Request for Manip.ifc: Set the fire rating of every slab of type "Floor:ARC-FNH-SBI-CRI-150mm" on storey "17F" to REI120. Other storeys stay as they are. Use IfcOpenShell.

First a look at what the model holds.

```python
import ifcopenshell
import ifcopenshell.util.element

model = ifcopenshell.open("Manip.ifc")
print(model.schema)
storey = next(s for s in model.by_type("IfcBuildingStorey") if s.Name == "17F")
slabs = [e for e in ifcopenshell.util.element.get_decomposition(storey) if e.is_a("IfcSlab")]
seen = {}
for e in slabs:
    element_type = ifcopenshell.util.element.get_type(e)
    key = (element_type.Name if element_type != e and element_type else None, ifcopenshell.util.element.get_pset(e, "Pset_SlabCommon", "FireRating"))
    seen[key] = seen.get(key, 0) + 1
for (name, value), count in sorted(seen.items(), key=str):
    print(count, "x", name, "|", value)
```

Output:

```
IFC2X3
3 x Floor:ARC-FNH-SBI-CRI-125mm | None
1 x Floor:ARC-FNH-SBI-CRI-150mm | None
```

```python
import ifcopenshell
import ifcopenshell.api.pset
import ifcopenshell.util.element

model = ifcopenshell.open("Manip.ifc")

storey = next(s for s in model.by_type("IfcBuildingStorey") if s.Name == "17F")
slabs = [e for e in ifcopenshell.util.element.get_decomposition(storey) if e.is_a("IfcSlab")]

count = 0
for e in slabs:
    element_type = ifcopenshell.util.element.get_type(e)
    if element_type in (None, e) or element_type.Name != "Floor:ARC-FNH-SBI-CRI-150mm":
        continue
    # add_pset returns the element's existing set when there is one.
    pset = ifcopenshell.api.pset.add_pset(model, product=e, name="Pset_SlabCommon")
    ifcopenshell.api.pset.edit_pset(model, pset=pset, properties={"FireRating": "REI120"})
    count += 1

print(count, "slabs updated")

model.write("Manip_rev.ifc")
```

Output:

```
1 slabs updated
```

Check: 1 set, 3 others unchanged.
